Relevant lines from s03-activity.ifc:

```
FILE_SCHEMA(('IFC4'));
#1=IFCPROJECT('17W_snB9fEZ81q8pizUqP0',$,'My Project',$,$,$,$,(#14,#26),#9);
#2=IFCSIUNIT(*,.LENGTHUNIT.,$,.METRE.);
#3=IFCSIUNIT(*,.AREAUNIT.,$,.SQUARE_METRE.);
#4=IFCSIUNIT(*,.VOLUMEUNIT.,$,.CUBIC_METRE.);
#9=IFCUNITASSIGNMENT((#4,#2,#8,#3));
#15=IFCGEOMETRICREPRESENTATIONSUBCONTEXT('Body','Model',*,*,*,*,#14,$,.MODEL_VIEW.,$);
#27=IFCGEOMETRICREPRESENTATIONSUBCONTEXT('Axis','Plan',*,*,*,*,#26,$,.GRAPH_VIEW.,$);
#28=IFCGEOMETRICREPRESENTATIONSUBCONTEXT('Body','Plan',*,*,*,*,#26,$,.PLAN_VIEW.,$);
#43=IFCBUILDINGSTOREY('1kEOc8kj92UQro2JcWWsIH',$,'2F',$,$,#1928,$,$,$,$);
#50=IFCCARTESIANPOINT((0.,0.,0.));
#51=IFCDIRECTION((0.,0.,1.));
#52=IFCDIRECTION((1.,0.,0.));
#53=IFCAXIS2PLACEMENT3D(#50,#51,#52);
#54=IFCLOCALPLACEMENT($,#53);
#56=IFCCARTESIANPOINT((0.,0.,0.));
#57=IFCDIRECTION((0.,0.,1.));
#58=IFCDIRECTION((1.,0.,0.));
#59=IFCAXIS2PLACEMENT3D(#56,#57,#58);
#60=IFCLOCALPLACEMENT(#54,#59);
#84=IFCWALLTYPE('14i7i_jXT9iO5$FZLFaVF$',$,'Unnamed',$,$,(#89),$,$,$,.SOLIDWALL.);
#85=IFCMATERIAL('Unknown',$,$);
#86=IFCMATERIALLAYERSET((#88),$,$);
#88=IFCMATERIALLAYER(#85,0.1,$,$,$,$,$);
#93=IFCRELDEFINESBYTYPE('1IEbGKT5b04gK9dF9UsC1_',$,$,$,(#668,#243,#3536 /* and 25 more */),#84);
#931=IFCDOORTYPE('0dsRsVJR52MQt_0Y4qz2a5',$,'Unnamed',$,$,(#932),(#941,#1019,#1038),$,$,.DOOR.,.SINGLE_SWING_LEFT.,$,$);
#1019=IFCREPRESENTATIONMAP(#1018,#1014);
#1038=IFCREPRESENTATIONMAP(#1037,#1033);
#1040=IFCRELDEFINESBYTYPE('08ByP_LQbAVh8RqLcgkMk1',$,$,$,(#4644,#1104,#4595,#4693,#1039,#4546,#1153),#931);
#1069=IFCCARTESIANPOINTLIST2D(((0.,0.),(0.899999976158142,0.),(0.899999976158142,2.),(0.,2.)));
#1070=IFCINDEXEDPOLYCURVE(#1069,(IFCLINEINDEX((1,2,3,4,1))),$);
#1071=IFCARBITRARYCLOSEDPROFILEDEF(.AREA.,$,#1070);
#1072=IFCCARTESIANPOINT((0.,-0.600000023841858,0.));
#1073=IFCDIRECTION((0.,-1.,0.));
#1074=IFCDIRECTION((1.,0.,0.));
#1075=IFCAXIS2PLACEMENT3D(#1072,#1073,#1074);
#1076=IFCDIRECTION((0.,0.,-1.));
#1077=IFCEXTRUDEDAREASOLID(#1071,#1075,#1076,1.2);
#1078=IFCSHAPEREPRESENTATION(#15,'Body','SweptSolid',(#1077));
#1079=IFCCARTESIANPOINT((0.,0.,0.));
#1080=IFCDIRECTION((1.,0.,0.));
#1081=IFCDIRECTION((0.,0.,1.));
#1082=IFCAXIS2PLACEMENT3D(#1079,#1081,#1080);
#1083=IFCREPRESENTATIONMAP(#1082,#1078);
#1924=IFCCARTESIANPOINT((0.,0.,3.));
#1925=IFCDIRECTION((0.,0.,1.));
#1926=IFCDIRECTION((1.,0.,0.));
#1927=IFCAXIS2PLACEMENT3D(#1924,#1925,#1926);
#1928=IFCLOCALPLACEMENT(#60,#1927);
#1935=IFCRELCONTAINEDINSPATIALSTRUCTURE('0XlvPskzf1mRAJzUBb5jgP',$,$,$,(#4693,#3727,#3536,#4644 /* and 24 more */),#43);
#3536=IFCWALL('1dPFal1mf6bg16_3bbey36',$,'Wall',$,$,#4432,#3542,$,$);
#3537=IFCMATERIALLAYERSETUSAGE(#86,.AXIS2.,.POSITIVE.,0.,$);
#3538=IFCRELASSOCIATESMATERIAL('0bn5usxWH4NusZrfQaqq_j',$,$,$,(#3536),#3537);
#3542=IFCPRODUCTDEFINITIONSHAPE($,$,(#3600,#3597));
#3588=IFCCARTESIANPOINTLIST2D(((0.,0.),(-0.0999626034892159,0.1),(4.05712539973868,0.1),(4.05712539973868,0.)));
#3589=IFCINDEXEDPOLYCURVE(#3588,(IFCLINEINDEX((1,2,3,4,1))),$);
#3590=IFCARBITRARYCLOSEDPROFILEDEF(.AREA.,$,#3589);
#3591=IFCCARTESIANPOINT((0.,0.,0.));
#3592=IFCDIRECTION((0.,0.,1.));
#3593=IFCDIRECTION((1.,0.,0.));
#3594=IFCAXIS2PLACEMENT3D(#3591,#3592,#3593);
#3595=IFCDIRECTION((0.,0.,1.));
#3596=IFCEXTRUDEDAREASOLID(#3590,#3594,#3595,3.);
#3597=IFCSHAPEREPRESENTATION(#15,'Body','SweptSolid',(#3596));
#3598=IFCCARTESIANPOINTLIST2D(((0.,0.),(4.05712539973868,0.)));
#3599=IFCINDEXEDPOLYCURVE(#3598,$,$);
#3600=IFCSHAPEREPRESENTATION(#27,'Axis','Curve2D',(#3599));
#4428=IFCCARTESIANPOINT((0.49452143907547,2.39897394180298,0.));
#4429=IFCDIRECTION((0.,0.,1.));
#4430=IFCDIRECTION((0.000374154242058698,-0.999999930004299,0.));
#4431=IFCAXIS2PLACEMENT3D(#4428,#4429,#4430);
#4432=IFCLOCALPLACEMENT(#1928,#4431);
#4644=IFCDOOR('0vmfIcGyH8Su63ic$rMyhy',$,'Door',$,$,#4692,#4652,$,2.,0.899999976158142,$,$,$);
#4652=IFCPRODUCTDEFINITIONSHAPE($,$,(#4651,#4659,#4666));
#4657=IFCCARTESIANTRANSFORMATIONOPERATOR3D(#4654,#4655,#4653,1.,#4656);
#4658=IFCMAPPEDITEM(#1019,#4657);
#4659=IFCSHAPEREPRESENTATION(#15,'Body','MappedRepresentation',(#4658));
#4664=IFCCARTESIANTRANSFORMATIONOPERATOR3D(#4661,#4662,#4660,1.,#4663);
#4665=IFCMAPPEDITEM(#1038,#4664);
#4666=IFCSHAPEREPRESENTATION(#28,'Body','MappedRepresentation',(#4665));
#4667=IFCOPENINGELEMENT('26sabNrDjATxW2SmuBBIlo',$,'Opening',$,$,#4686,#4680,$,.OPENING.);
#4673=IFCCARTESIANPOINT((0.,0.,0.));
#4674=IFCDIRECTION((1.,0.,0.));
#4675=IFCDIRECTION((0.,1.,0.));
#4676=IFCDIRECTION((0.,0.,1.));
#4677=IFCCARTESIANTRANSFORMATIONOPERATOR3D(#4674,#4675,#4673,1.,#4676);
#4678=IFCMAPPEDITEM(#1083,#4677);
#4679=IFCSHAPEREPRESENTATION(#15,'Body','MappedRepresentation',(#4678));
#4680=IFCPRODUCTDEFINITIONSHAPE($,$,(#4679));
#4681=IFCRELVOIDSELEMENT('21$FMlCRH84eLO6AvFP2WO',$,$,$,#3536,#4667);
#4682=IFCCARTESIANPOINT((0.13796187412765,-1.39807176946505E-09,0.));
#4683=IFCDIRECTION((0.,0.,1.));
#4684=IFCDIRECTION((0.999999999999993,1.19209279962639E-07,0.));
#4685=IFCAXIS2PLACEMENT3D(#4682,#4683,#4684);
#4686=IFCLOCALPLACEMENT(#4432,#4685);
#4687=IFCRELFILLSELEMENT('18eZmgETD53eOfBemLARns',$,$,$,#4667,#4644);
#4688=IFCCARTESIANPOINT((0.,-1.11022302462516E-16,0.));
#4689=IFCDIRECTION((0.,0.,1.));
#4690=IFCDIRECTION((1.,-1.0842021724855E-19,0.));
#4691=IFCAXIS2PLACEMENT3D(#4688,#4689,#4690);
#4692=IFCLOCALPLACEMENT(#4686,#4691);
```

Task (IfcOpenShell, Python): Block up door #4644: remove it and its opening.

```python
import ifcopenshell
import ifcopenshell.api.feature
import ifcopenshell.api.root
import ifcopenshell.geom
import ifcopenshell.util.shape

model = ifcopenshell.open("s03-activity.ifc")
settings = ifcopenshell.geom.settings()


def volume(element):
    """Net volume in cubic metres, openings subtracted."""
    shape = ifcopenshell.geom.create_shape(settings, element)
    return ifcopenshell.util.shape.get_volume(shape.geometry)


door = model.by_id(4644)
opening = door.FillsVoids[0].RelatingOpeningElement
wall = opening.VoidsElements[0].RelatingBuildingElement
before = volume(wall)

ifcopenshell.api.root.remove_product(model, product=door)
ifcopenshell.api.feature.remove_feature(model, feature=opening)

after = volume(wall)

print(f"wall volume {before:.3f} -> {after:.3f} m3")

model.write("s03-activity_updated.ifc")
```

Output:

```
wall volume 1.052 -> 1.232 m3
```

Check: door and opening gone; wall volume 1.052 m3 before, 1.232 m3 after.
